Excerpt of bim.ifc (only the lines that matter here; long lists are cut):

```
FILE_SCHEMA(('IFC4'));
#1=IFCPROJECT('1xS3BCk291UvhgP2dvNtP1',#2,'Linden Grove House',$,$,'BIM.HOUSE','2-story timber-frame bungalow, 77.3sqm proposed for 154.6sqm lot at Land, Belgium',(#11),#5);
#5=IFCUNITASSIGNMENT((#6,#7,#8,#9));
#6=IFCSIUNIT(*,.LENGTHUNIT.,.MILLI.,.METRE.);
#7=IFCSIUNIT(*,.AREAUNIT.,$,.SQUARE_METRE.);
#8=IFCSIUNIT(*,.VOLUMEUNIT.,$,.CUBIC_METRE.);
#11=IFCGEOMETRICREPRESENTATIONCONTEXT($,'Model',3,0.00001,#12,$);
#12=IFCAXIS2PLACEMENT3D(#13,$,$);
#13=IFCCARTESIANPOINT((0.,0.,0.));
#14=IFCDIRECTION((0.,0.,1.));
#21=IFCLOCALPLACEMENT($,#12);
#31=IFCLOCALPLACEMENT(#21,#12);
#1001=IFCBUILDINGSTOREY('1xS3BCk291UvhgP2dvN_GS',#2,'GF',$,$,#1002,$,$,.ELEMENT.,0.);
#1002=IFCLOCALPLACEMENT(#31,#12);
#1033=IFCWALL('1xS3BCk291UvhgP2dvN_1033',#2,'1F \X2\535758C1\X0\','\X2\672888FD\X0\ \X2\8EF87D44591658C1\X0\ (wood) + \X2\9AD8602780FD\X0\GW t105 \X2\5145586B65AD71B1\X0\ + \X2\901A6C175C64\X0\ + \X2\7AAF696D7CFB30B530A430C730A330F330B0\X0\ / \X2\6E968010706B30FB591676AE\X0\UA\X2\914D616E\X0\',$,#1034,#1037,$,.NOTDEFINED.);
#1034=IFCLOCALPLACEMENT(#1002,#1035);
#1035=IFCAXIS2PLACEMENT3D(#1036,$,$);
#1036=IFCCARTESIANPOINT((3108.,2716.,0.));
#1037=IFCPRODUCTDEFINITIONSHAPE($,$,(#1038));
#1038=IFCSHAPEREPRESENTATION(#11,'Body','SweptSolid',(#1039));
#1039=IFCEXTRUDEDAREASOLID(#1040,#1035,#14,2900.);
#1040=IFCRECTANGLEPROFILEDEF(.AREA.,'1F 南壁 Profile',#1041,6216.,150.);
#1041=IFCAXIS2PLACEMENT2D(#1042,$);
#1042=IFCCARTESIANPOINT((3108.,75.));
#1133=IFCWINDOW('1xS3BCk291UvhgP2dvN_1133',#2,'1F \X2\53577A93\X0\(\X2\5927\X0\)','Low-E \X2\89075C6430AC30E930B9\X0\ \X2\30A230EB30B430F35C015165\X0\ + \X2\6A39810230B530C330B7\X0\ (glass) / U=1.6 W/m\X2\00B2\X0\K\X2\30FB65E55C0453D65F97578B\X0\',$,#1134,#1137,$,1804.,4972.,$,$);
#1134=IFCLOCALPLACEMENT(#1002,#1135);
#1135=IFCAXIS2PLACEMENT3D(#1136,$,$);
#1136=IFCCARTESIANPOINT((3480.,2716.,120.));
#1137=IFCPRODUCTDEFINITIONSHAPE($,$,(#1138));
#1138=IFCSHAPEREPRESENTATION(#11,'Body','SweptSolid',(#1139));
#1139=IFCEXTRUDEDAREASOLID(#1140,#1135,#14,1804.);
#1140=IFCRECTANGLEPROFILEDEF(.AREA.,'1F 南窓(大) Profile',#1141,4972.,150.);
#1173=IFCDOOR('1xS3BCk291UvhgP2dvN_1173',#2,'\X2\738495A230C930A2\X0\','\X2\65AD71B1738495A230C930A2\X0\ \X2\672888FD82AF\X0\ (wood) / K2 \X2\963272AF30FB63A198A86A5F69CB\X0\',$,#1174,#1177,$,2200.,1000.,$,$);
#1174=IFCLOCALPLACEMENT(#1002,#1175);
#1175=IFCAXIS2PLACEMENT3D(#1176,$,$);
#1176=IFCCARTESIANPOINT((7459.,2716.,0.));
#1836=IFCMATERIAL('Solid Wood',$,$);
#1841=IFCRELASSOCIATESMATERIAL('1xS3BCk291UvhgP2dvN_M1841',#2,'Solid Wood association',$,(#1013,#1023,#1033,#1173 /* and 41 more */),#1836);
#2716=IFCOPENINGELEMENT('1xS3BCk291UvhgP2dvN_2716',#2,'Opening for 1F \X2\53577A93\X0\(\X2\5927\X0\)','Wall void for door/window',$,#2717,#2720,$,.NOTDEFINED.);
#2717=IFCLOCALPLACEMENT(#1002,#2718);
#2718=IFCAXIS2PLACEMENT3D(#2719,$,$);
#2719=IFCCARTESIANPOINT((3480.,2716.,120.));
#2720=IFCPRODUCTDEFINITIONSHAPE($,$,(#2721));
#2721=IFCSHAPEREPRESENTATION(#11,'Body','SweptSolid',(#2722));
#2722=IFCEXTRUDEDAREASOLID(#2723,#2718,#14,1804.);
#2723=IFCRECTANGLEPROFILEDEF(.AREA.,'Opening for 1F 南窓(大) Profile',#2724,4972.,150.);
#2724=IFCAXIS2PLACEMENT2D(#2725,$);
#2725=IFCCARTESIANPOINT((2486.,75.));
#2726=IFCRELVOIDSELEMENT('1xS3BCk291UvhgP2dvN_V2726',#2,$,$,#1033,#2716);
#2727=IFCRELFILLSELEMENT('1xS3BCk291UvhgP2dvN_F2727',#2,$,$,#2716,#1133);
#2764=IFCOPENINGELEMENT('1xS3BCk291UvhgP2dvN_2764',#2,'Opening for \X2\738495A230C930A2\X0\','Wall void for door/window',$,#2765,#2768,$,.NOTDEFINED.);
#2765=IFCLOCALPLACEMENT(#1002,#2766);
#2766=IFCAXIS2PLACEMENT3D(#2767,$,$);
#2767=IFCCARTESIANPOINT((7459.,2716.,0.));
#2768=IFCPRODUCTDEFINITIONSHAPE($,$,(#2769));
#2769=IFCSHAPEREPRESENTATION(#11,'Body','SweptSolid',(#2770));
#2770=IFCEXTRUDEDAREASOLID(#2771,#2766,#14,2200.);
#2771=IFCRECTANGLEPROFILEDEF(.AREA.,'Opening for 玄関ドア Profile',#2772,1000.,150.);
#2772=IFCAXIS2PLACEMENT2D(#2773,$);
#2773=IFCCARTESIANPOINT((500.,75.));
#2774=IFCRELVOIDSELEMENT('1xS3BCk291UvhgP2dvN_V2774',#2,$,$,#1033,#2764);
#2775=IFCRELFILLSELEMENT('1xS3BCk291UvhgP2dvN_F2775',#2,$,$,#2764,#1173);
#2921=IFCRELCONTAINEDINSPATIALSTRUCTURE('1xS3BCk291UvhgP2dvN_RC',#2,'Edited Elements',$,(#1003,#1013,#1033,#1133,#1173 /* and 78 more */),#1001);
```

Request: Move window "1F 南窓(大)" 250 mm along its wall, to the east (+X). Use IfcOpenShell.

```python
import ifcopenshell
import ifcopenshell.api.geometry
import ifcopenshell.util.placement
import ifcopenshell.util.unit

model = ifcopenshell.open("bim.ifc")
unit_scale = ifcopenshell.util.unit.calculate_unit_scale(model)

window = model.by_guid("1xS3BCk291UvhgP2dvN_1133")
opening = window.FillsVoids[0].RelatingOpeningElement
wall = opening.VoidsElements[0].RelatingBuildingElement

wall_matrix = ifcopenshell.util.placement.get_local_placement(wall.ObjectPlacement)
shift = wall_matrix[:3, 0] * 0.25 / unit_scale
before = ifcopenshell.util.placement.get_local_placement(window.ObjectPlacement)[:3, 3].copy()

# The window is not placed relative to its opening, so move both.
for product in (opening, window):
    matrix = ifcopenshell.util.placement.get_local_placement(product.ObjectPlacement)
    matrix[:3, 3] += shift
    ifcopenshell.api.geometry.edit_object_placement(model, product=product, matrix=matrix, is_si=False)

after = ifcopenshell.util.placement.get_local_placement(window.ObjectPlacement)[:3, 3]
print("window moved by", (after - before).round(3) + 0.0)

model.write("bim_updated.ifc")
```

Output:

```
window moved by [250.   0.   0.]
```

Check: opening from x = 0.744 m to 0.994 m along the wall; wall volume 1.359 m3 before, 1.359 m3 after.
